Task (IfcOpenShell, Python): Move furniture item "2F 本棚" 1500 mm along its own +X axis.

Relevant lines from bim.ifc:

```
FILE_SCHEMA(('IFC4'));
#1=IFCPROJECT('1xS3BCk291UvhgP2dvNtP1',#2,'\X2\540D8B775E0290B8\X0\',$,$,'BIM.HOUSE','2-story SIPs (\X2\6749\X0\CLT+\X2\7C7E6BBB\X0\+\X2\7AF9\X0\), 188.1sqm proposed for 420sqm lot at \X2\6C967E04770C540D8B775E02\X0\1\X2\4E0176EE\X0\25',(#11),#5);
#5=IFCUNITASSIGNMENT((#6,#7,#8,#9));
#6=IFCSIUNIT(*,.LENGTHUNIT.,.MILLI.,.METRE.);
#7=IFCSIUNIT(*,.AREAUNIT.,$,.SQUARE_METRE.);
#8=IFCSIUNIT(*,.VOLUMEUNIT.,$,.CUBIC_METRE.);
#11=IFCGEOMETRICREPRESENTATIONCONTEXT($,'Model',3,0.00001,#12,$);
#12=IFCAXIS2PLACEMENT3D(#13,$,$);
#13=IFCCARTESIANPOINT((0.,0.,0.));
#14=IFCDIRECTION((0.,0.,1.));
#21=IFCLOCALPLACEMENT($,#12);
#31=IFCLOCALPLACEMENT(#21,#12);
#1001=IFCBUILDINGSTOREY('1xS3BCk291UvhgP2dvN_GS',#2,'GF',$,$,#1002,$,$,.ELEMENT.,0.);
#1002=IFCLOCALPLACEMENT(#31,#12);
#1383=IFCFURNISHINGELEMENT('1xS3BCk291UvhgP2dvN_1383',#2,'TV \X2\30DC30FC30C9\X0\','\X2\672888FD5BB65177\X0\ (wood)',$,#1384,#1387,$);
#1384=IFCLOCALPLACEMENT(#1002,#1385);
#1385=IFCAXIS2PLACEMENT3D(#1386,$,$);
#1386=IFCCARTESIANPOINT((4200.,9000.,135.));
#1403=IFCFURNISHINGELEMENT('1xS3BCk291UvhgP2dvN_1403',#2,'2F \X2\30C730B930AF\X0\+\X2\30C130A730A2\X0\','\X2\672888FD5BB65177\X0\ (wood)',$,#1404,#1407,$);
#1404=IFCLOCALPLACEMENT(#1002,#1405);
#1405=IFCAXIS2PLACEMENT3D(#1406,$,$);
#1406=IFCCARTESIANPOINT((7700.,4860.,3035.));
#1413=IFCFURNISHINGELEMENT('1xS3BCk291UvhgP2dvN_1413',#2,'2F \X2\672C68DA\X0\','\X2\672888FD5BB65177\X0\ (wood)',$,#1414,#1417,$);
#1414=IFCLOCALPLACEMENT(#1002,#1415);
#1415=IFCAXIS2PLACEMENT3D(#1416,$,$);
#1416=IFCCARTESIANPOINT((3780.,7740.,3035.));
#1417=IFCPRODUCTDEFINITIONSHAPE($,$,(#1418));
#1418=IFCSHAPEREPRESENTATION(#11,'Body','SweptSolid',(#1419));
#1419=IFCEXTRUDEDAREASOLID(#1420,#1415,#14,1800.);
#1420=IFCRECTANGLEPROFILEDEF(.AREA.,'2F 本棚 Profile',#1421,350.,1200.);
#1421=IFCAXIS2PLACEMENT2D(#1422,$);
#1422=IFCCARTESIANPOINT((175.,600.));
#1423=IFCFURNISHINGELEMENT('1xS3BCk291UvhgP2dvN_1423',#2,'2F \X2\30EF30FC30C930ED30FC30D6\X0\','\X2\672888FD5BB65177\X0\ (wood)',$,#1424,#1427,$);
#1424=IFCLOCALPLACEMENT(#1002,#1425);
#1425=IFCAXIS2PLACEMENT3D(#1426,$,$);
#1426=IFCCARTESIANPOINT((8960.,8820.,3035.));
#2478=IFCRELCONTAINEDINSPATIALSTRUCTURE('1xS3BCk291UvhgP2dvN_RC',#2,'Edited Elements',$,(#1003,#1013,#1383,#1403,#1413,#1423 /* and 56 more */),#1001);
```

```python
import ifcopenshell
import ifcopenshell.api.geometry
import ifcopenshell.util.placement

model = ifcopenshell.open("bim.ifc")

item = model.by_id(1413)
matrix = ifcopenshell.util.placement.get_local_placement(item.ObjectPlacement)
matrix[:3, 3] += matrix[:3, 0] * 1500.0
ifcopenshell.api.geometry.edit_object_placement(model, product=item, matrix=matrix, is_si=False)

print(ifcopenshell.util.placement.get_local_placement(item.ObjectPlacement).round(3) + 0.0)

model.write("bim_edited.ifc")
```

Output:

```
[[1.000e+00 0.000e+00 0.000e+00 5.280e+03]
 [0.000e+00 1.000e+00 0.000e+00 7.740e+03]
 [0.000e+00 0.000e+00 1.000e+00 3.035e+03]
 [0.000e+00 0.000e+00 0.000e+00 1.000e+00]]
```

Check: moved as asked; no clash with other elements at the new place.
